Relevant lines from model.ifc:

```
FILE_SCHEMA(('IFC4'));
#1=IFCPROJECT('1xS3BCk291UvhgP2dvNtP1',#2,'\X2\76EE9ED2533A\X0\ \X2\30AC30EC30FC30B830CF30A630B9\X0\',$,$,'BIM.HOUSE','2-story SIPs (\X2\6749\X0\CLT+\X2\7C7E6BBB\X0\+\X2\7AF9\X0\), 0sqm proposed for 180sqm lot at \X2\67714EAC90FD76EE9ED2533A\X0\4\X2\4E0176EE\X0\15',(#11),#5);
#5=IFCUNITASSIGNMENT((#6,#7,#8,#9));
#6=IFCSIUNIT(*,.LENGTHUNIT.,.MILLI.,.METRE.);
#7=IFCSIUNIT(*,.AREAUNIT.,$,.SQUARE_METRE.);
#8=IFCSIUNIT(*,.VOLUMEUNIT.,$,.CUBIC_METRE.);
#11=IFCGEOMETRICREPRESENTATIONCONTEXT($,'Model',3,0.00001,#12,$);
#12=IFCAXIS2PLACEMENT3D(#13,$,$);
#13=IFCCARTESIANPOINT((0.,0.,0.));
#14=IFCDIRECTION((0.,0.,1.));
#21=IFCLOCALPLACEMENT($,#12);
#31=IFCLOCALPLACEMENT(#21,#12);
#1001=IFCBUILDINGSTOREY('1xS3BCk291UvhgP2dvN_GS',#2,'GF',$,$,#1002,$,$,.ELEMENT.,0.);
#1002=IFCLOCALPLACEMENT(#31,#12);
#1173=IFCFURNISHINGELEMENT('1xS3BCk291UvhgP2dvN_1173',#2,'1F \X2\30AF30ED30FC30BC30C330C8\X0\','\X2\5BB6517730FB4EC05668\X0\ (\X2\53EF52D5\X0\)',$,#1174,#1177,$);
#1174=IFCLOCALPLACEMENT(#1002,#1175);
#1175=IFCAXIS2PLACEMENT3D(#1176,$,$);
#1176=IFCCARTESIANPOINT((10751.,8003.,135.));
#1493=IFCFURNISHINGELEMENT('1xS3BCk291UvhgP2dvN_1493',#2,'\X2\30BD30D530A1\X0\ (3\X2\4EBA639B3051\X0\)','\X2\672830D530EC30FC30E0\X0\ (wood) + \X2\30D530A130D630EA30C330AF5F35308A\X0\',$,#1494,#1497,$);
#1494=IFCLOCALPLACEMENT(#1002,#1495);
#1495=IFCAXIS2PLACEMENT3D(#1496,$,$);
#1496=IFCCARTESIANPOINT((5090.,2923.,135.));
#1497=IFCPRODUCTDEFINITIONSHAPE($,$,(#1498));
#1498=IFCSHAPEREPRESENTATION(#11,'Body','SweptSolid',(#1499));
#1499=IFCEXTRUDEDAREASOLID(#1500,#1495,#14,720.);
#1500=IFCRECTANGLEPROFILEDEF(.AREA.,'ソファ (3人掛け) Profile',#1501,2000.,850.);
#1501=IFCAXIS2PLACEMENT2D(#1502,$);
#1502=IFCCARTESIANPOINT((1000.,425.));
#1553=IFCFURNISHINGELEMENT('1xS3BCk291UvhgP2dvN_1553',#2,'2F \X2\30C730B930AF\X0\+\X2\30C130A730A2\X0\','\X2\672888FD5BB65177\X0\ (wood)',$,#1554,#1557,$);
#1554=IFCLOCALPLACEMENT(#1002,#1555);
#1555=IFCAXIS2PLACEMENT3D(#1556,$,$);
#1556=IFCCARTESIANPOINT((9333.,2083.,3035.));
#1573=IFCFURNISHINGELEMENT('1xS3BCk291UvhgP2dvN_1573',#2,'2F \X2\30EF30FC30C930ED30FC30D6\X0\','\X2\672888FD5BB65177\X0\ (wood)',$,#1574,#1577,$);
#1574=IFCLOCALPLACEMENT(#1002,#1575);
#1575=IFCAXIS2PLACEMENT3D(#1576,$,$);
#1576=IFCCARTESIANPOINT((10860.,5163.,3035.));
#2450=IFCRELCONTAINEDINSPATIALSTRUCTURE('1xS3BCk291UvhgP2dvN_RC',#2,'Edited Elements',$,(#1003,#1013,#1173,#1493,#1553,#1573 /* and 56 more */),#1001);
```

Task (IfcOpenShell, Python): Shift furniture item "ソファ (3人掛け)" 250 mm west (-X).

```python
import ifcopenshell
import ifcopenshell.api.geometry
import ifcopenshell.util.placement

model = ifcopenshell.open("model.ifc")

item = model.by_guid("1xS3BCk291UvhgP2dvN_1493")
matrix = ifcopenshell.util.placement.get_local_placement(item.ObjectPlacement)
matrix[0, 3] -= 250.0
ifcopenshell.api.geometry.edit_object_placement(model, product=item, matrix=matrix, is_si=False)

print(ifcopenshell.util.placement.get_local_placement(item.ObjectPlacement).round(3) + 0.0)

model.write("model_edited.ifc")
```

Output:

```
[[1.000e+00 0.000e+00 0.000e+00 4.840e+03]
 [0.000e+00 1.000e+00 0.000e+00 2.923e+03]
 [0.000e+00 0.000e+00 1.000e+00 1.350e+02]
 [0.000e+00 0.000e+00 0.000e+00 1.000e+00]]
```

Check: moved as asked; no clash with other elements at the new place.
